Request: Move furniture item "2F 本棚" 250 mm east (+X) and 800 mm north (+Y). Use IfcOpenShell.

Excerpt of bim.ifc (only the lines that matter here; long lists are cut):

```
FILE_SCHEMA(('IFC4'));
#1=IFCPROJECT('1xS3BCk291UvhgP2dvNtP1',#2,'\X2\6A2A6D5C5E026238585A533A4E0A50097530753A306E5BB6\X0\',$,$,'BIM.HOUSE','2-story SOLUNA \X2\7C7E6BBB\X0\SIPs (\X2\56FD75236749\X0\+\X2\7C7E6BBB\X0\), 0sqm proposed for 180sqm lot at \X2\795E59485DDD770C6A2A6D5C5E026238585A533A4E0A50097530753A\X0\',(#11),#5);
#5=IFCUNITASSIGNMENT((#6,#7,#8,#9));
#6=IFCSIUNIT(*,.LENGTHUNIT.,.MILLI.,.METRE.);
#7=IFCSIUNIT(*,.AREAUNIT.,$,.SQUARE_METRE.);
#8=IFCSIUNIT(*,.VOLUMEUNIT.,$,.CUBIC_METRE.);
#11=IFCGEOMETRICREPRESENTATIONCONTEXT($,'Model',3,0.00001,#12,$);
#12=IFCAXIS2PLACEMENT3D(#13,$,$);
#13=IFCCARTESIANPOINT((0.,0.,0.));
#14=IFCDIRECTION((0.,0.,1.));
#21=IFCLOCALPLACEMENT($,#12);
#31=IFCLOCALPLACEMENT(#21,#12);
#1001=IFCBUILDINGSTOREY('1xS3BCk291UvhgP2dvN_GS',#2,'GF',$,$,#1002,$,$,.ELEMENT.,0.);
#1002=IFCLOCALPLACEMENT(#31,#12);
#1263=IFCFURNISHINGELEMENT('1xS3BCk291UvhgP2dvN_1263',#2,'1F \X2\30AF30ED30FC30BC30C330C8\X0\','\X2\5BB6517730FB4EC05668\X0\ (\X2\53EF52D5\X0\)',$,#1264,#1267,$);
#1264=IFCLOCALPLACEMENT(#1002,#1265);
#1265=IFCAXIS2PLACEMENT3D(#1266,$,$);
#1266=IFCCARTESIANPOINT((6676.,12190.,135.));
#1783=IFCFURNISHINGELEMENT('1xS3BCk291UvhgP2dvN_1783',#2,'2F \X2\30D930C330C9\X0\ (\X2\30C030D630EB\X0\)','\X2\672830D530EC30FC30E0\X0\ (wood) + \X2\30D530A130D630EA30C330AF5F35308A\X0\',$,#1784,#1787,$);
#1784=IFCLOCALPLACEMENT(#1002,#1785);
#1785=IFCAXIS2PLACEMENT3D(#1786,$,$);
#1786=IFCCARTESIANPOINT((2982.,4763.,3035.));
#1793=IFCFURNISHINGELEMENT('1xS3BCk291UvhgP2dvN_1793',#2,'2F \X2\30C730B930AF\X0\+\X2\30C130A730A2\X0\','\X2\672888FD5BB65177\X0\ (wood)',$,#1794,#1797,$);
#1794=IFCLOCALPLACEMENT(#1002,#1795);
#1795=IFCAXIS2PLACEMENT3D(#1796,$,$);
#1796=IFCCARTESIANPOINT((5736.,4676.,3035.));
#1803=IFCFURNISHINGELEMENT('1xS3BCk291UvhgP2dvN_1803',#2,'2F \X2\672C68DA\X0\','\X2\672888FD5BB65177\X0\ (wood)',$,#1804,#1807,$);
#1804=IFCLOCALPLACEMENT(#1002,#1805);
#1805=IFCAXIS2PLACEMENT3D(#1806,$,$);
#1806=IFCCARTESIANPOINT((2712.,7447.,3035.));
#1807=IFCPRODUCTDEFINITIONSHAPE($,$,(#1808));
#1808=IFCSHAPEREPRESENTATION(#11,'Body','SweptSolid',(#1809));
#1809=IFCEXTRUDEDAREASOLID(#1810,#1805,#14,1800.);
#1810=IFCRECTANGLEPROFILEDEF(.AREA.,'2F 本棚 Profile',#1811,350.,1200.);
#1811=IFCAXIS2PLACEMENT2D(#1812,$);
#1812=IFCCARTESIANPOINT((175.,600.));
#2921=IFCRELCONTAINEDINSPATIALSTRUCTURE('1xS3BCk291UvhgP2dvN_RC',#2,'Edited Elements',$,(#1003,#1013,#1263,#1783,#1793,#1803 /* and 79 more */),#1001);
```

```python
import ifcopenshell
import ifcopenshell.api.geometry
import ifcopenshell.util.placement
import ifcopenshell.util.unit

model = ifcopenshell.open("bim.ifc")
unit_scale = ifcopenshell.util.unit.calculate_unit_scale(model)

item = model.by_guid("1xS3BCk291UvhgP2dvN_1803")
matrix = ifcopenshell.util.placement.get_local_placement(item.ObjectPlacement)
matrix[0, 3] += 0.25 / unit_scale
matrix[1, 3] += 0.8 / unit_scale
ifcopenshell.api.geometry.edit_object_placement(model, product=item, matrix=matrix, is_si=False)

print(ifcopenshell.util.placement.get_local_placement(item.ObjectPlacement).round(3) + 0.0)

model.write("bim_edited.ifc")
```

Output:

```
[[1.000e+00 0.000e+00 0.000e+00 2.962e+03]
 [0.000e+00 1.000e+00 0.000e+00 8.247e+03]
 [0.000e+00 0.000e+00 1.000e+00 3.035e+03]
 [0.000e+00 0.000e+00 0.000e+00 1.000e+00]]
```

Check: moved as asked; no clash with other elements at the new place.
